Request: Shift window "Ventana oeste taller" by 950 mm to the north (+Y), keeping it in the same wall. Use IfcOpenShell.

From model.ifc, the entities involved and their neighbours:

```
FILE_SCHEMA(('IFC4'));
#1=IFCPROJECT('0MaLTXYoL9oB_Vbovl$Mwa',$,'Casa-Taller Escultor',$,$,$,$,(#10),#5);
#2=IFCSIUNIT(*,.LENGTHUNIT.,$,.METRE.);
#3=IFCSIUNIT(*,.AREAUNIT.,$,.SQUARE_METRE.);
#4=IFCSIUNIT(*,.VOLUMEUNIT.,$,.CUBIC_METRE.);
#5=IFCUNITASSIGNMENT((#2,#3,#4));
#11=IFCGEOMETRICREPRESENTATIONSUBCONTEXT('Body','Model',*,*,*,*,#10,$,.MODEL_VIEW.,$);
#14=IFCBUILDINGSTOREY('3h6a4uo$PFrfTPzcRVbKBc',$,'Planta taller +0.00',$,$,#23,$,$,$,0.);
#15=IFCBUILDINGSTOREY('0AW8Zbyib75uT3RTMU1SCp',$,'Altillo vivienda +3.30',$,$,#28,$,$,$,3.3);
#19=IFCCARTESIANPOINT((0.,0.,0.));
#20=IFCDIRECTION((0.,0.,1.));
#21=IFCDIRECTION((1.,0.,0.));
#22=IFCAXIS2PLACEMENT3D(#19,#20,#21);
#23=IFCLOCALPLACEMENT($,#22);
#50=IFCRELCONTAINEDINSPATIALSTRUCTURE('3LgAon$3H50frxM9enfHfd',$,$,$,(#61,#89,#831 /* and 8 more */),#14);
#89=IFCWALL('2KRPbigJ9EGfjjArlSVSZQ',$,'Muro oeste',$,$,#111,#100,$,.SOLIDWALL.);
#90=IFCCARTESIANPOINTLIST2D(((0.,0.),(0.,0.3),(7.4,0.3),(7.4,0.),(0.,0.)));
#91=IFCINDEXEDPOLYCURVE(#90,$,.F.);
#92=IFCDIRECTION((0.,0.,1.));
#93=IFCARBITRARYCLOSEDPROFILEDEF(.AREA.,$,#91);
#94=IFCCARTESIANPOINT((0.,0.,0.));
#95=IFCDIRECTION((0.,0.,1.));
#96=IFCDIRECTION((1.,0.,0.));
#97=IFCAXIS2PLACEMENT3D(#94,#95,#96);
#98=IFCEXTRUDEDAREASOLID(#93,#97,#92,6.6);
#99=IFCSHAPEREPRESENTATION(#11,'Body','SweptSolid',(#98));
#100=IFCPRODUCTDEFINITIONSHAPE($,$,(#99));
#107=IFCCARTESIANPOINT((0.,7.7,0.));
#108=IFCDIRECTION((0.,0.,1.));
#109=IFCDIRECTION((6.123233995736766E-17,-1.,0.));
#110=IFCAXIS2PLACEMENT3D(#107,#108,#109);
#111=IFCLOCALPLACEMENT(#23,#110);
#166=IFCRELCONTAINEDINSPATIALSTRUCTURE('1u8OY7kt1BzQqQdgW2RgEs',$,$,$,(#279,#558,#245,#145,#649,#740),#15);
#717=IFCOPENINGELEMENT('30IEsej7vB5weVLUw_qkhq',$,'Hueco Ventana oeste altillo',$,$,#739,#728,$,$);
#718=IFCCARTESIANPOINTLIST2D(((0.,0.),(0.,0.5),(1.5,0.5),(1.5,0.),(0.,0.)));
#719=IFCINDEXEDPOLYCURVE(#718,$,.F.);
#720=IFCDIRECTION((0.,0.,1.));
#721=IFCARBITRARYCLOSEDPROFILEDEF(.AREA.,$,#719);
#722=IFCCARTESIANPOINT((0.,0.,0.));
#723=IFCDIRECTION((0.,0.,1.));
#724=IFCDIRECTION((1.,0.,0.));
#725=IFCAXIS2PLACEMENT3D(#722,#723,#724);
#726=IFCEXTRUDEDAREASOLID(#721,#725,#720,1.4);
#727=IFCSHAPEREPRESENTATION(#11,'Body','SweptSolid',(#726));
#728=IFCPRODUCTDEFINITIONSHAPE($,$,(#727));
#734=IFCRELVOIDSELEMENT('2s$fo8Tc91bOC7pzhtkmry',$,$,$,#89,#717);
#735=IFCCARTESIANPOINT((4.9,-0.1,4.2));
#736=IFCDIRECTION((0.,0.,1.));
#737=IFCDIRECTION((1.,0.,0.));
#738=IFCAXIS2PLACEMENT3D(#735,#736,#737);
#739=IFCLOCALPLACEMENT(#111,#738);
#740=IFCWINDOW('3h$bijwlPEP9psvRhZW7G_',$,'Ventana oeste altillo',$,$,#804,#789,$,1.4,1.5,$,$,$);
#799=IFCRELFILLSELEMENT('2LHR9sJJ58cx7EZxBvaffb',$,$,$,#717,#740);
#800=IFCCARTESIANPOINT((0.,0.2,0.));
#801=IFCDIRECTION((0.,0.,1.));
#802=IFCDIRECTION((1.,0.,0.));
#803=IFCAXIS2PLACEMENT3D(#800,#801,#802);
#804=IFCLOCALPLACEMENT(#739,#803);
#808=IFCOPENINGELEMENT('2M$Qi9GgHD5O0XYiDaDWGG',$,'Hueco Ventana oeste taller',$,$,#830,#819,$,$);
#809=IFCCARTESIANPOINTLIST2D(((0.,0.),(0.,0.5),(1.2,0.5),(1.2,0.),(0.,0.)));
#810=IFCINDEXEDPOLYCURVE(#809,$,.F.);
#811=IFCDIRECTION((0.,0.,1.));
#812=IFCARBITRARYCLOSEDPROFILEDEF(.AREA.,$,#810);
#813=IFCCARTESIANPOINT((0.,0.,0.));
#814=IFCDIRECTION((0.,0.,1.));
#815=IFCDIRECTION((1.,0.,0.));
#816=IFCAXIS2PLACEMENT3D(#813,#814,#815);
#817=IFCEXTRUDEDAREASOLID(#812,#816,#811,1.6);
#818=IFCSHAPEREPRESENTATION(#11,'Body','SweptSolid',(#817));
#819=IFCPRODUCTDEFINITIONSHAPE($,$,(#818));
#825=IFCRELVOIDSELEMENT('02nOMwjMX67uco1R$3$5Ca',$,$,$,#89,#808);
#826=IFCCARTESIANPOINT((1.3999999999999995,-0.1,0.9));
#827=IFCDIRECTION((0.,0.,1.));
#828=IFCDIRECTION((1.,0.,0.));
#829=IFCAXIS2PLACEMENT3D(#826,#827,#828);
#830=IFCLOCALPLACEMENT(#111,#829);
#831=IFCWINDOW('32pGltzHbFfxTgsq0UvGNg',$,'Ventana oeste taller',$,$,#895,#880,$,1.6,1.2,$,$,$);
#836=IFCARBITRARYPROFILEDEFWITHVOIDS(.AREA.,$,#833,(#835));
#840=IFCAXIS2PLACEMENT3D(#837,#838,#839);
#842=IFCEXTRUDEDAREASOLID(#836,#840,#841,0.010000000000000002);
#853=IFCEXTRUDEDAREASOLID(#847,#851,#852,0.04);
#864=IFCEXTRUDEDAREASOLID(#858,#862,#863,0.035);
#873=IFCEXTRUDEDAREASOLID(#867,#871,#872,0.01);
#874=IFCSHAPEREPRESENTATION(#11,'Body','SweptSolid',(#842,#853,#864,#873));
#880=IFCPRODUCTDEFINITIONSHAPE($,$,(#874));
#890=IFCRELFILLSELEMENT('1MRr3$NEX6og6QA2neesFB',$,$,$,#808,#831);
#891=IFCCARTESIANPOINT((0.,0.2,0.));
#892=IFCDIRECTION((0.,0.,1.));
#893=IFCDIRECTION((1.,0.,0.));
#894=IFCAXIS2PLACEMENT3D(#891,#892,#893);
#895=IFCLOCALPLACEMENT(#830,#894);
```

```python
import ifcopenshell
import ifcopenshell.api.geometry
import ifcopenshell.util.placement

model = ifcopenshell.open("model.ifc")

window = model.by_guid("32pGltzHbFfxTgsq0UvGNg")
opening = window.FillsVoids[0].RelatingOpeningElement
wall = opening.VoidsElements[0].RelatingBuildingElement

wall_matrix = ifcopenshell.util.placement.get_local_placement(wall.ObjectPlacement)
shift = wall_matrix[:3, 0] * -0.95
before = ifcopenshell.util.placement.get_local_placement(window.ObjectPlacement)[:3, 3].copy()

# The window is placed relative to its opening, so it follows when the opening moves.
matrix = ifcopenshell.util.placement.get_local_placement(opening.ObjectPlacement)
matrix[:3, 3] += shift
ifcopenshell.api.geometry.edit_object_placement(
    model, product=opening, matrix=matrix, is_si=False, should_transform_children=True
)

after = ifcopenshell.util.placement.get_local_placement(window.ObjectPlacement)[:3, 3]
print("window moved by", (after - before).round(3) + 0.0)

model.write("model-out.ifc")
```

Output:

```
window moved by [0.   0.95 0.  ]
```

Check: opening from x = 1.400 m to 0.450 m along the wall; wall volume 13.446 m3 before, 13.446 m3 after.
